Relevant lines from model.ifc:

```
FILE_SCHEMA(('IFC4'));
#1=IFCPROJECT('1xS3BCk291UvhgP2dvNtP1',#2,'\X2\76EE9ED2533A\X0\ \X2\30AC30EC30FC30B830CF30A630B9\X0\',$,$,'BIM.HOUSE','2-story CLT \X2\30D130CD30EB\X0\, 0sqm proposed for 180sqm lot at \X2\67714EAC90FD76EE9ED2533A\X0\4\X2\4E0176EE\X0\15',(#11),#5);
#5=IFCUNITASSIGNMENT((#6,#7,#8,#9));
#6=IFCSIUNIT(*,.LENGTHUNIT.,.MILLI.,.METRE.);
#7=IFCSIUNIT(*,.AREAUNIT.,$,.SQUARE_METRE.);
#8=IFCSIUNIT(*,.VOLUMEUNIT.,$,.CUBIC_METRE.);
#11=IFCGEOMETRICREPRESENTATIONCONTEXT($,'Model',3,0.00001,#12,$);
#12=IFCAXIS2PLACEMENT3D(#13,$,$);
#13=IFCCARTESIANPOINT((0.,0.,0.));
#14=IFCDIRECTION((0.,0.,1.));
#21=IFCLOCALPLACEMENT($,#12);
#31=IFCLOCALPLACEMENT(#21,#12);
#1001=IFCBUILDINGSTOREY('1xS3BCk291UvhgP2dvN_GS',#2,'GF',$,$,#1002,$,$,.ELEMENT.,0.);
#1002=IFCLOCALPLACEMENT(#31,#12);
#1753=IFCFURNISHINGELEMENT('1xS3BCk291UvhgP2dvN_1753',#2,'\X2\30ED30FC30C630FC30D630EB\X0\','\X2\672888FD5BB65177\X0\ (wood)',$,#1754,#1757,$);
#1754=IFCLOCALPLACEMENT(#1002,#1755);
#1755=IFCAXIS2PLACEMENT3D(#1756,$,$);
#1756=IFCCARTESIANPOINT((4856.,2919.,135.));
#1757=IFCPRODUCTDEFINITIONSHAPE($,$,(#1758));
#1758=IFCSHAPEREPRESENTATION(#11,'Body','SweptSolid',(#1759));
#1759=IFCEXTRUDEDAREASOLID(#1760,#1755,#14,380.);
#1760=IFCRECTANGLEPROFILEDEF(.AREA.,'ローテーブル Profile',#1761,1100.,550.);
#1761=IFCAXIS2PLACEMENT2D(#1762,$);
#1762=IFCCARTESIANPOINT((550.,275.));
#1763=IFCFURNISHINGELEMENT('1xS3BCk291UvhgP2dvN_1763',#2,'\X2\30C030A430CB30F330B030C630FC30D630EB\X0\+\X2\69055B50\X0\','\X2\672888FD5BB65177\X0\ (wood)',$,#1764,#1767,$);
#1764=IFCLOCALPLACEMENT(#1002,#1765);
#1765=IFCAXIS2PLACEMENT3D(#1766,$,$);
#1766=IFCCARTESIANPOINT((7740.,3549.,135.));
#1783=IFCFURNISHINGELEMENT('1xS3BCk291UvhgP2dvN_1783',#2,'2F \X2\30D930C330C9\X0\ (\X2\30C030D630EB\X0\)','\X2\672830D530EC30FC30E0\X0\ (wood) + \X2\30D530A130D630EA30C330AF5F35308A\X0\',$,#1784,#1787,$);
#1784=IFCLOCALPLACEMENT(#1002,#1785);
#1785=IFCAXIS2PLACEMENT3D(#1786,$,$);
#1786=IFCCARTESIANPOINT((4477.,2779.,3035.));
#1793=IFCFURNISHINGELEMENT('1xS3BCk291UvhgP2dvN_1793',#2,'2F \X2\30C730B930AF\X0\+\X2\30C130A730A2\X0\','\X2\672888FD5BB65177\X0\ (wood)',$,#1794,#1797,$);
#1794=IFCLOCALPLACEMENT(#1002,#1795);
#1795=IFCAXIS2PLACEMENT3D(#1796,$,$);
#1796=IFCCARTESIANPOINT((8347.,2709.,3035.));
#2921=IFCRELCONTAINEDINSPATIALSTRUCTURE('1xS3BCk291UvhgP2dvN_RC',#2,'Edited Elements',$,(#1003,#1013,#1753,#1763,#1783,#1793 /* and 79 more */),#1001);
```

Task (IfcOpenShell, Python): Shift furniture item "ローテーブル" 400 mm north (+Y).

```python
import ifcopenshell
import ifcopenshell.api.geometry
import ifcopenshell.util.placement
import ifcopenshell.util.unit

model = ifcopenshell.open("model.ifc")
unit_scale = ifcopenshell.util.unit.calculate_unit_scale(model)

item = model.by_id(1753)
matrix = ifcopenshell.util.placement.get_local_placement(item.ObjectPlacement)
matrix[1, 3] += 0.4 / unit_scale
ifcopenshell.api.geometry.edit_object_placement(model, product=item, matrix=matrix, is_si=False)

print(ifcopenshell.util.placement.get_local_placement(item.ObjectPlacement).round(3) + 0.0)

model.write("model_rev.ifc")
```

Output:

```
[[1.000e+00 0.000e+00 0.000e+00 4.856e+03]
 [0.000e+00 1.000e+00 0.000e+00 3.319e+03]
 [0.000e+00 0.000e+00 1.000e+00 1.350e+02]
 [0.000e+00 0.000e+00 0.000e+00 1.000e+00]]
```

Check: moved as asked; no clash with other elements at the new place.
